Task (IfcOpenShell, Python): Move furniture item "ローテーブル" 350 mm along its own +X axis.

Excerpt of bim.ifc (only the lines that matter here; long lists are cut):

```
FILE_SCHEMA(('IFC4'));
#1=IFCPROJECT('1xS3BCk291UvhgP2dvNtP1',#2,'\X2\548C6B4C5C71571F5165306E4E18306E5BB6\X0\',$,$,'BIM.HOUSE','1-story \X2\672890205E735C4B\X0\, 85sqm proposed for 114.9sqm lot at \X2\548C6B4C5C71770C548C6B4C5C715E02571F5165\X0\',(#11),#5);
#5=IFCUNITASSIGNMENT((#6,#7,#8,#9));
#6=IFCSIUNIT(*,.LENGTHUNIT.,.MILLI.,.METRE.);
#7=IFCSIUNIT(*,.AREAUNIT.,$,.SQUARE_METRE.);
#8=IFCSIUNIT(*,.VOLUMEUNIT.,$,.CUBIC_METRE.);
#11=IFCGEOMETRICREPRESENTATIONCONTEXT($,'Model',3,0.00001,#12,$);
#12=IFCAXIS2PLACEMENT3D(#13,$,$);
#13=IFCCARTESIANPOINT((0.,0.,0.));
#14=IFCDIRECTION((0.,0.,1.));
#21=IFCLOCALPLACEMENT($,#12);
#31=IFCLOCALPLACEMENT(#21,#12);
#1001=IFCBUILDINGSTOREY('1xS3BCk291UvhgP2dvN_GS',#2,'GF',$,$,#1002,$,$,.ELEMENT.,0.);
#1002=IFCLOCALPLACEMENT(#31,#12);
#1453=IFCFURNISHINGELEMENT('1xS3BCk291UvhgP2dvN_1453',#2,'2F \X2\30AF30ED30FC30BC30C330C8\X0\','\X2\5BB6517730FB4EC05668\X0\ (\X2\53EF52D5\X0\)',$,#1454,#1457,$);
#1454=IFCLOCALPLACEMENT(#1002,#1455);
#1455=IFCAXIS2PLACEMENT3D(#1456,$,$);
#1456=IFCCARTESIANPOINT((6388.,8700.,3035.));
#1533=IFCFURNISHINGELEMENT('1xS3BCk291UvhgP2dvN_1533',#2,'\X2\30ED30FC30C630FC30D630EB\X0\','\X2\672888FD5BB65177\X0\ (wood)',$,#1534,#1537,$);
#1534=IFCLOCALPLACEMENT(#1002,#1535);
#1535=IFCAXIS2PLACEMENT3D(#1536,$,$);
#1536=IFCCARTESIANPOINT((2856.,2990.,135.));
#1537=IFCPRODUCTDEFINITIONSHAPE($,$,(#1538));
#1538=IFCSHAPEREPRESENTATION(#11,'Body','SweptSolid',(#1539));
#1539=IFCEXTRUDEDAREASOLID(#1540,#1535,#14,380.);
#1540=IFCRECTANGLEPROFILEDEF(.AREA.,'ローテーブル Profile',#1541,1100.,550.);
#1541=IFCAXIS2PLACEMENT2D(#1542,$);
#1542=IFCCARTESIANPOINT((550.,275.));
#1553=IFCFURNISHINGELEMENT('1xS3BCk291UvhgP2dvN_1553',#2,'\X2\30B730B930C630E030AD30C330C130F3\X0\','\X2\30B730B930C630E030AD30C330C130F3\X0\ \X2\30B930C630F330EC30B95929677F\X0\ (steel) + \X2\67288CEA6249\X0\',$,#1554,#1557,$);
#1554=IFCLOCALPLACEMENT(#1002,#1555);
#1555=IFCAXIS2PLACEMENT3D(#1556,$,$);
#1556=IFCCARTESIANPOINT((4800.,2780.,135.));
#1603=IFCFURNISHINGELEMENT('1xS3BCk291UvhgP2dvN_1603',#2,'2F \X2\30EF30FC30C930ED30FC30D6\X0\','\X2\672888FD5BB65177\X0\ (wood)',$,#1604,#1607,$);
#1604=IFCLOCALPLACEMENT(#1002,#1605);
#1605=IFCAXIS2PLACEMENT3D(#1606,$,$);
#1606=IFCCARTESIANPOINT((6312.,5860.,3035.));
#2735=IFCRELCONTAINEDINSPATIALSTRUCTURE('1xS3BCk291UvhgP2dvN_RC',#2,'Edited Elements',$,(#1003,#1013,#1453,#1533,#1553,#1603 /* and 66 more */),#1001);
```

```python
import ifcopenshell
import ifcopenshell.api.geometry
import ifcopenshell.util.placement

model = ifcopenshell.open("bim.ifc")

item = model.by_id(1533)
matrix = ifcopenshell.util.placement.get_local_placement(item.ObjectPlacement)
matrix[:3, 3] += matrix[:3, 0] * 350.0
ifcopenshell.api.geometry.edit_object_placement(model, product=item, matrix=matrix, is_si=False)

print(ifcopenshell.util.placement.get_local_placement(item.ObjectPlacement).round(3) + 0.0)

model.write("bim_updated.ifc")
```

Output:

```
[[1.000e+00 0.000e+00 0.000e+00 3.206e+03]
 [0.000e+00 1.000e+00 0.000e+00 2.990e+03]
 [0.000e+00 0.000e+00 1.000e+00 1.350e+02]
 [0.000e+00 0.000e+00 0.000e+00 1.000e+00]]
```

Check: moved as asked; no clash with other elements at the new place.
